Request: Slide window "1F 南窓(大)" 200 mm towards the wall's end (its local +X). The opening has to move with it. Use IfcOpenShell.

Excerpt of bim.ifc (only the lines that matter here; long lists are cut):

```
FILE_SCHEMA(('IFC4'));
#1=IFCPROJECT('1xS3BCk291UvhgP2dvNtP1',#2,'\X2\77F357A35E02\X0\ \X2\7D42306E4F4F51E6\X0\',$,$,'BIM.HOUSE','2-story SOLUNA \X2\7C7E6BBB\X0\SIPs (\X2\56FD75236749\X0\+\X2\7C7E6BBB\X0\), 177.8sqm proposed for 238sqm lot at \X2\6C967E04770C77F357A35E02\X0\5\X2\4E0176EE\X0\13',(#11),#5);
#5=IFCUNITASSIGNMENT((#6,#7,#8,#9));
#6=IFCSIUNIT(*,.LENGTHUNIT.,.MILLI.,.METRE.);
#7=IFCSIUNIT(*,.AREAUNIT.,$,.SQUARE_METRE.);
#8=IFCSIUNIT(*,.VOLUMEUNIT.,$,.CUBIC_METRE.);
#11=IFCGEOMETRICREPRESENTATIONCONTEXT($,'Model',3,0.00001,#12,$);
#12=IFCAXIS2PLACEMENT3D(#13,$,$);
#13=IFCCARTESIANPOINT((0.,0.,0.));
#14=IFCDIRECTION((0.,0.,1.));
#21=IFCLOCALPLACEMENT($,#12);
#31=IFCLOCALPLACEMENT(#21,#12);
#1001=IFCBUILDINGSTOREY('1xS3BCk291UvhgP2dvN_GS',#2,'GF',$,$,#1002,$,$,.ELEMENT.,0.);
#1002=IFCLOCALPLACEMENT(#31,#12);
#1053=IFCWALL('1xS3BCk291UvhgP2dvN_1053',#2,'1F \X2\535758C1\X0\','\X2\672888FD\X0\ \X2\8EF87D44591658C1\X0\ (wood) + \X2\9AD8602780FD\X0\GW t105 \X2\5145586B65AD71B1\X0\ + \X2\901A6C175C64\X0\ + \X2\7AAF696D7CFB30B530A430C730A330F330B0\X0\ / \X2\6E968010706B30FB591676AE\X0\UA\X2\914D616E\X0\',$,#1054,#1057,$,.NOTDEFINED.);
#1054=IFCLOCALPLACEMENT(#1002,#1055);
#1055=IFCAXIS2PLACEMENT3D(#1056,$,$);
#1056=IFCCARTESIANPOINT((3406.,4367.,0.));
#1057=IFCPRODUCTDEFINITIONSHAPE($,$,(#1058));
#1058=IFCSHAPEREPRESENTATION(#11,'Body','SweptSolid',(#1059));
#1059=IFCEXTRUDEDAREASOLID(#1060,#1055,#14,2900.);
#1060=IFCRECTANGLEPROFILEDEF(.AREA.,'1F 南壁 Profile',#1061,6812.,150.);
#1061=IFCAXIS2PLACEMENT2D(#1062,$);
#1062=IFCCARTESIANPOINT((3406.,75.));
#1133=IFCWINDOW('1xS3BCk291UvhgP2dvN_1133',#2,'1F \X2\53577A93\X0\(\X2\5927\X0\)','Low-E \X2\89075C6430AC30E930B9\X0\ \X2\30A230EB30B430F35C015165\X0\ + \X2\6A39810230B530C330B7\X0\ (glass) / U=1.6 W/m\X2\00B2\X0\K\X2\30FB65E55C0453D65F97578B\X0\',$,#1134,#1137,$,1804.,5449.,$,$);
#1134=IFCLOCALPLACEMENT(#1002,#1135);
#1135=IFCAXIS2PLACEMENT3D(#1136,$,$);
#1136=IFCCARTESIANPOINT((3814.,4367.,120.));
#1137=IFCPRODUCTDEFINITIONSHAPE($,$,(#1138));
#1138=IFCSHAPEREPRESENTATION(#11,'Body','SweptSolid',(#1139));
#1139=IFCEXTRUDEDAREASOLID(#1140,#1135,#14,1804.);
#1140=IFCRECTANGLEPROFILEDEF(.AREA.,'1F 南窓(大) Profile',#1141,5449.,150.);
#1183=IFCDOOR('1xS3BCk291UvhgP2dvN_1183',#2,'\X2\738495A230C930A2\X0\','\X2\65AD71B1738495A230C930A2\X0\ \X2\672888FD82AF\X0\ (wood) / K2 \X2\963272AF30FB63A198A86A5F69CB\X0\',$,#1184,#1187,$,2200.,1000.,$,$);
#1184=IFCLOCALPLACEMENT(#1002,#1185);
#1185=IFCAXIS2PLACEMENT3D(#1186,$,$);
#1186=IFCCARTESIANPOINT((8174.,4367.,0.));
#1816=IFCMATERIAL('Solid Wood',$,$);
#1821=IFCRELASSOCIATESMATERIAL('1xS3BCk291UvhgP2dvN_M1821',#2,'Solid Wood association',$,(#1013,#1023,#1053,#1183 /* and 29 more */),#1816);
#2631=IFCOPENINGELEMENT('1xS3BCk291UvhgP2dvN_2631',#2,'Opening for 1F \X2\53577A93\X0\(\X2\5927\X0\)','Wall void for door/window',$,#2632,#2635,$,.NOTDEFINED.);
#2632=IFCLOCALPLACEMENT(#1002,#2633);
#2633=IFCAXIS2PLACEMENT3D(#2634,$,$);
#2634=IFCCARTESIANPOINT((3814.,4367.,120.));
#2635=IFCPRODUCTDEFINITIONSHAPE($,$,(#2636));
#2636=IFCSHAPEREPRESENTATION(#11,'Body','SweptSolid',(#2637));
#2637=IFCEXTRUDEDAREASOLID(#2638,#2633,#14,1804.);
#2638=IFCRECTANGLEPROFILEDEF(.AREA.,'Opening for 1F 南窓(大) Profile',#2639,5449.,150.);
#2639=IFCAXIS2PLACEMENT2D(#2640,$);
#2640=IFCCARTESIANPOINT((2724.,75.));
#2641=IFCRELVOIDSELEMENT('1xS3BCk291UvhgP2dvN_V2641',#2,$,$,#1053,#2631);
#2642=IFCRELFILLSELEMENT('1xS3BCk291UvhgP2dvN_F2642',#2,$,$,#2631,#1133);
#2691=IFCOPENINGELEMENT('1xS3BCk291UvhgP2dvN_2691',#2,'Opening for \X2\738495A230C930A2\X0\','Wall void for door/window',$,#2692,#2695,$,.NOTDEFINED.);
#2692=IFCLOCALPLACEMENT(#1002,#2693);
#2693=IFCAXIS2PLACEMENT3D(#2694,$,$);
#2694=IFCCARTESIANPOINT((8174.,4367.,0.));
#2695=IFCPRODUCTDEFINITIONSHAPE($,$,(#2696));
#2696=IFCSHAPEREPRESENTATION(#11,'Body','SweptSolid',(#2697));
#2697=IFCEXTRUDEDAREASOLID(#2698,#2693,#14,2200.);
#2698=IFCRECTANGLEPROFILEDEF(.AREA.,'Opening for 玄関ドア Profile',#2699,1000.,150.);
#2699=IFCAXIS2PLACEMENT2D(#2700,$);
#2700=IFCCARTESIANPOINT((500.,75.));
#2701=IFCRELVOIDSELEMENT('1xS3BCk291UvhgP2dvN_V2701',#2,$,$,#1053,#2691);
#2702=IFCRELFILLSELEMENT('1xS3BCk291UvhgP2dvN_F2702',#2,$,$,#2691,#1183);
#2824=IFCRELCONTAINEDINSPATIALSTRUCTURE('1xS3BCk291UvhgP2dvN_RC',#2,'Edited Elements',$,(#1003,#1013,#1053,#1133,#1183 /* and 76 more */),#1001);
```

```python
import ifcopenshell
import ifcopenshell.api.geometry
import ifcopenshell.util.placement
import ifcopenshell.util.unit

model = ifcopenshell.open("bim.ifc")
unit_scale = ifcopenshell.util.unit.calculate_unit_scale(model)

window = model.by_id(1133)
opening = window.FillsVoids[0].RelatingOpeningElement
wall = opening.VoidsElements[0].RelatingBuildingElement

wall_matrix = ifcopenshell.util.placement.get_local_placement(wall.ObjectPlacement)
shift = wall_matrix[:3, 0] * 0.2 / unit_scale
before = ifcopenshell.util.placement.get_local_placement(window.ObjectPlacement)[:3, 3].copy()

# The window is not placed relative to its opening, so move both.
for product in (opening, window):
    matrix = ifcopenshell.util.placement.get_local_placement(product.ObjectPlacement)
    matrix[:3, 3] += shift
    ifcopenshell.api.geometry.edit_object_placement(model, product=product, matrix=matrix, is_si=False)

after = ifcopenshell.util.placement.get_local_placement(window.ObjectPlacement)[:3, 3]
print("window moved by", (after - before).round(3) + 0.0)

model.write("bim_v2.ifc")
```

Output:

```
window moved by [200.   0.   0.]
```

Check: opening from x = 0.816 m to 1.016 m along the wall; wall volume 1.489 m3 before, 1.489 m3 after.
